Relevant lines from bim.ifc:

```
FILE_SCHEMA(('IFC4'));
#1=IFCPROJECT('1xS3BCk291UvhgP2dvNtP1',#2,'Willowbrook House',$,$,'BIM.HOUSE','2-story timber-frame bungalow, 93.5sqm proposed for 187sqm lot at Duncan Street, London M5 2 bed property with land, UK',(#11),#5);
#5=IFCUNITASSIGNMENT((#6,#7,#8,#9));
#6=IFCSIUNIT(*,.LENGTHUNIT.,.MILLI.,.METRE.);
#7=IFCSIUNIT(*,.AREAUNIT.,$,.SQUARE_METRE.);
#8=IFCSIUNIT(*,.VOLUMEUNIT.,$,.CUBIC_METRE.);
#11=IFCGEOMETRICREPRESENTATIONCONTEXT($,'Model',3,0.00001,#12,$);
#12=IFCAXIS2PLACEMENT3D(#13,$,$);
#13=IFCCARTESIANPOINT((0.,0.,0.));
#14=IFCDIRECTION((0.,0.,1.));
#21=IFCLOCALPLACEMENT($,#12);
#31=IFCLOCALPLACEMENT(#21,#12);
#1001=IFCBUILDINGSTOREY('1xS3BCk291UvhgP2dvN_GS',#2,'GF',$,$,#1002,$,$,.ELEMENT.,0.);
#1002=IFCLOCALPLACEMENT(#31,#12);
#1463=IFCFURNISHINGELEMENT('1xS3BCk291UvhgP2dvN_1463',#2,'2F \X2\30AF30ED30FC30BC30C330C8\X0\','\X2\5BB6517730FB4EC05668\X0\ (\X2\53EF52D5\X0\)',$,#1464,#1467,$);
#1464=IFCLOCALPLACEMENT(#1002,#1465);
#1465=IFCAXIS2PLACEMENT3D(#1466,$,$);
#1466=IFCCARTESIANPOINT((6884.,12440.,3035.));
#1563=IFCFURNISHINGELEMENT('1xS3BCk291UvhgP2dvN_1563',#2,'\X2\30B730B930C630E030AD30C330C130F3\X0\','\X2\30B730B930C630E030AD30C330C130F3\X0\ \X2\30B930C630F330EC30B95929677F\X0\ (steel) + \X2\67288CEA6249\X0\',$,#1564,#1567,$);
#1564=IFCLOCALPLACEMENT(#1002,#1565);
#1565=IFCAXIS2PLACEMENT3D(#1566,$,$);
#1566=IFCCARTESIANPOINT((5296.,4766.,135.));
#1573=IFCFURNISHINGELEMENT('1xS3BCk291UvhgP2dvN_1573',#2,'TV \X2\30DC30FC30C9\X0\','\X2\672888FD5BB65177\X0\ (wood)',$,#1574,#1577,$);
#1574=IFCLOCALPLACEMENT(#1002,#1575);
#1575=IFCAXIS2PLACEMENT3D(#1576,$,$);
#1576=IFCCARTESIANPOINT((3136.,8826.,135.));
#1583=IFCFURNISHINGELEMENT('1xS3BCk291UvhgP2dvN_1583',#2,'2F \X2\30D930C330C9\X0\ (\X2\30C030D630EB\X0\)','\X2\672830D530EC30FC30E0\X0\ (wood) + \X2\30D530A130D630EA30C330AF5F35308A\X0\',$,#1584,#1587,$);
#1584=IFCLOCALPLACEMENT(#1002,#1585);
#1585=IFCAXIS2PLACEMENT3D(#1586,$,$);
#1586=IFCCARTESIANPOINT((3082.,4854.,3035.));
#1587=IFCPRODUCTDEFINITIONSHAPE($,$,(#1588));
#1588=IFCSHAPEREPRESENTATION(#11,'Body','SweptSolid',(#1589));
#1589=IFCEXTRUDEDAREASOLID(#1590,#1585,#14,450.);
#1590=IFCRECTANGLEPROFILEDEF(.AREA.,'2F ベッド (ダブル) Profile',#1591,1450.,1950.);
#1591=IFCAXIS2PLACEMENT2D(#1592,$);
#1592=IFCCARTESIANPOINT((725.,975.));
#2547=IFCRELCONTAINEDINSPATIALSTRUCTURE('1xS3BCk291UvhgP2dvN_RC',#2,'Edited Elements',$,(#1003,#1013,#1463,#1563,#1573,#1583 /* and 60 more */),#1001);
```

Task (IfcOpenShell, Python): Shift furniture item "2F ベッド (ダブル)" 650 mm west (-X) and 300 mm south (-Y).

```python
import ifcopenshell
import ifcopenshell.api.geometry
import ifcopenshell.util.placement
import ifcopenshell.util.unit

model = ifcopenshell.open("bim.ifc")
unit_scale = ifcopenshell.util.unit.calculate_unit_scale(model)

item = model.by_guid("1xS3BCk291UvhgP2dvN_1583")
matrix = ifcopenshell.util.placement.get_local_placement(item.ObjectPlacement)
matrix[0, 3] -= 0.65 / unit_scale
matrix[1, 3] -= 0.3 / unit_scale
ifcopenshell.api.geometry.edit_object_placement(model, product=item, matrix=matrix, is_si=False)

print(ifcopenshell.util.placement.get_local_placement(item.ObjectPlacement).round(3) + 0.0)

model.write("bim_edited.ifc")
```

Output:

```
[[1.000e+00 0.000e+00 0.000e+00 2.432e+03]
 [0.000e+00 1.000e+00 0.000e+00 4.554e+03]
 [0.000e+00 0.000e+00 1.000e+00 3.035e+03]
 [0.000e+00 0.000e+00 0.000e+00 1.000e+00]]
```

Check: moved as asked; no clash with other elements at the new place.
